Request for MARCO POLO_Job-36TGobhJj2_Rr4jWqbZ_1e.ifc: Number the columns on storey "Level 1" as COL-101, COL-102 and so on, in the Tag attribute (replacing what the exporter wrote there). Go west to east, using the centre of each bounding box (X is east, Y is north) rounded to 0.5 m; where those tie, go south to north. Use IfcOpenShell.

First a look at what the model holds.

```python
import ifcopenshell
import ifcopenshell.util.element
import ifcopenshell.util.placement

model = ifcopenshell.open("MARCO POLO_Job-36TGobhJj2_Rr4jWqbZ_1e.ifc")
print(model.schema)
storey = next(s for s in model.by_type("IfcBuildingStorey") if s.Name == "Level 1")
columns = [e for e in ifcopenshell.util.element.get_decomposition(storey) if e.is_a("IfcColumn")]
for e in sorted(columns, key=lambda e: e.id()):
    origin = ifcopenshell.util.placement.get_local_placement(e.ObjectPlacement)[:3, 3]
    print(e.id(), e.Tag, e.Name, origin.round(2) + 0.0, sep=" | ")
```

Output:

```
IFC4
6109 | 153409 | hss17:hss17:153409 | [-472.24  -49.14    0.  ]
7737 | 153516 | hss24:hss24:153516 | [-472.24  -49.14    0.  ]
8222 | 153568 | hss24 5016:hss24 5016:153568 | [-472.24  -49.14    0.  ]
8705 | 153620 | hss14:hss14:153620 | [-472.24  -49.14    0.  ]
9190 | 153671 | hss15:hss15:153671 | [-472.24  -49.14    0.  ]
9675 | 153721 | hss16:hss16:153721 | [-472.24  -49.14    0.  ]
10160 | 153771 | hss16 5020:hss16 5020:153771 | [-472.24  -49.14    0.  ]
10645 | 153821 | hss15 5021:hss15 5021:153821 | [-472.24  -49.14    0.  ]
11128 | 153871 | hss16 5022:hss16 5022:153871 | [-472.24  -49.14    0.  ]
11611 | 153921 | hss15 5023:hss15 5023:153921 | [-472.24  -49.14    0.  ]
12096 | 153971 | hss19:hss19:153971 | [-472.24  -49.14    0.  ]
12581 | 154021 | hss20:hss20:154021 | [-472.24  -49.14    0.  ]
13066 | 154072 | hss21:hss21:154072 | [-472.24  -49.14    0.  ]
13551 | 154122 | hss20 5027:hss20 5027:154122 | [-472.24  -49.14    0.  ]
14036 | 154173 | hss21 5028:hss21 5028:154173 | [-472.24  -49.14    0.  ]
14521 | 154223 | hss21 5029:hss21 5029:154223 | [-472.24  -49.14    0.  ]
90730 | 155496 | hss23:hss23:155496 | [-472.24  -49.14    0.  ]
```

```python
import ifcopenshell
import ifcopenshell.geom
import ifcopenshell.util.element
import ifcopenshell.util.shape

model = ifcopenshell.open("MARCO POLO_Job-36TGobhJj2_Rr4jWqbZ_1e.ifc")
settings = ifcopenshell.geom.settings()
settings.set("use-world-coords", True)


def centre(element):
    shape = ifcopenshell.geom.create_shape(settings, element)
    return ifcopenshell.util.shape.get_bbox_centroid(shape.geometry)


storey = next(s for s in model.by_type("IfcBuildingStorey") if s.Name == "Level 1")
columns = [e for e in ifcopenshell.util.element.get_decomposition(storey) if e.is_a("IfcColumn")]

# Insertion points can sit at a corner or the storey origin, so sort by the geometry (in metres).
centres = {e: centre(e) for e in columns}
columns.sort(key=lambda e: (round(centres[e][0] / 0.5), centres[e][1]))

for i, e in enumerate(columns, start=1):
    number = f"COL-1{i:02d}"
    e.Tag = number
    print(e.id(), number)

model.write("MARCO POLO_Job-36TGobhJj2_Rr4jWqbZ_1e_v2.ifc")
```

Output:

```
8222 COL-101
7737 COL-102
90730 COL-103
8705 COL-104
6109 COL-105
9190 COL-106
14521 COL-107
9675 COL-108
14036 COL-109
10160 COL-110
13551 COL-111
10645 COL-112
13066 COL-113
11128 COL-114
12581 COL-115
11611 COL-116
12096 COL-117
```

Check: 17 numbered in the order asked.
